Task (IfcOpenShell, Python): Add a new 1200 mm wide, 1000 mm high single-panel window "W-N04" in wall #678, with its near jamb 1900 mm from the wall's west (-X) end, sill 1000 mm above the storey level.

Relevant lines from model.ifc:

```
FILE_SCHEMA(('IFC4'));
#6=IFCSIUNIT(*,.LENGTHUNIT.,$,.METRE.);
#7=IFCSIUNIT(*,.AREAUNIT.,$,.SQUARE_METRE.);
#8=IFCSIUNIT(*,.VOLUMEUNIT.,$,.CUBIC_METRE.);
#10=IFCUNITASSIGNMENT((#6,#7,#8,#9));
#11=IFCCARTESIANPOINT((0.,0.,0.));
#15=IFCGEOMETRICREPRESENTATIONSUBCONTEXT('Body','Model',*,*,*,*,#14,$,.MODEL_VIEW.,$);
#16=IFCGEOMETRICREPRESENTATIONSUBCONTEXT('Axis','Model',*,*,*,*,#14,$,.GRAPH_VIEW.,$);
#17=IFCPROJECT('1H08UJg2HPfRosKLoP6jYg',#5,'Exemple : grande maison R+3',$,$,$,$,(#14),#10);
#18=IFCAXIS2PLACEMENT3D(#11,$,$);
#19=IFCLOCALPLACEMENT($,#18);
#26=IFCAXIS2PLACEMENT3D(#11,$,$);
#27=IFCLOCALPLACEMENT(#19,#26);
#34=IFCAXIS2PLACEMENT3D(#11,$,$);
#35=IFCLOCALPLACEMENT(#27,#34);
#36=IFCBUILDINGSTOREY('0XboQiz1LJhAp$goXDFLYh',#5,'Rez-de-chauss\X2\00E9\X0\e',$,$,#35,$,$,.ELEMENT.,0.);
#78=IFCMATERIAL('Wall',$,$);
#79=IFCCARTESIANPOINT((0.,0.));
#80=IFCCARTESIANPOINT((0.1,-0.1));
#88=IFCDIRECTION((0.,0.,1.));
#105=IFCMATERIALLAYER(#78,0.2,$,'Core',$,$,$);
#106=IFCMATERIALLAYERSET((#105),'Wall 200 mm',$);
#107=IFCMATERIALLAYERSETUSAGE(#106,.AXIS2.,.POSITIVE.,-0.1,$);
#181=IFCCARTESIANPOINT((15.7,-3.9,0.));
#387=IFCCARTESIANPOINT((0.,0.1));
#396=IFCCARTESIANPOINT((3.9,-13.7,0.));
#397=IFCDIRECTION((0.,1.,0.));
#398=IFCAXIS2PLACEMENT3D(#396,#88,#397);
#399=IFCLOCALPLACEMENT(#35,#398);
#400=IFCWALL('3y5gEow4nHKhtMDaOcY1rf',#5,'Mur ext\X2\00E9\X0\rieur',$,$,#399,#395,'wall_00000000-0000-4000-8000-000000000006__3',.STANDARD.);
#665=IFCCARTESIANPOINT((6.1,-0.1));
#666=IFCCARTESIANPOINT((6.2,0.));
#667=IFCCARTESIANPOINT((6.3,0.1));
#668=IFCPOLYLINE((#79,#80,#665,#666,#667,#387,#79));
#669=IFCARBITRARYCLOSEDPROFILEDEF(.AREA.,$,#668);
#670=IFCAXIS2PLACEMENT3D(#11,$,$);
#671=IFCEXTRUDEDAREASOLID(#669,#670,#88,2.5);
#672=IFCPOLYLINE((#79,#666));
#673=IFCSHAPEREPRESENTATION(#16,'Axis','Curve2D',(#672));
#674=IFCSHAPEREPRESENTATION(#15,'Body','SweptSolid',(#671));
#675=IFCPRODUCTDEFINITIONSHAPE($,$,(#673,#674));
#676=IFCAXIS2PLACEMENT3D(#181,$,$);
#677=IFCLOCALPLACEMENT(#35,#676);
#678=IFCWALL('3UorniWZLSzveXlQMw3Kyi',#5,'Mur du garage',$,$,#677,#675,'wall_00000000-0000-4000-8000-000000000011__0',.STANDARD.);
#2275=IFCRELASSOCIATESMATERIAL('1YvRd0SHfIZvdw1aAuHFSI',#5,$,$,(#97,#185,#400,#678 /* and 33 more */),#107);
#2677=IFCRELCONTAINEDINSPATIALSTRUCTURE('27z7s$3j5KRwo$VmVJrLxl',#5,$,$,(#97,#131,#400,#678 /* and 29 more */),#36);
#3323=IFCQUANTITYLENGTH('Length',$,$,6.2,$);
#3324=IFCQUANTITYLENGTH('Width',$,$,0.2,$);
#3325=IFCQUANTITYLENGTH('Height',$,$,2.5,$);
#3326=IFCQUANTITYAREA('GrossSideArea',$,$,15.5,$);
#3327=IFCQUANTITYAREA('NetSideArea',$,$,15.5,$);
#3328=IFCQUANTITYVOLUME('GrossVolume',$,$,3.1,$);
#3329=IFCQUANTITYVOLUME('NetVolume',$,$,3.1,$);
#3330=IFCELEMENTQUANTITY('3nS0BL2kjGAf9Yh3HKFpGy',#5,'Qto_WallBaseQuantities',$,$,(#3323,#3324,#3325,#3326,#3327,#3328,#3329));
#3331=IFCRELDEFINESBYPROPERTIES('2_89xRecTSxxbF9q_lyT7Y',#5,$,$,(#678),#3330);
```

```python
import numpy as np
import ifcopenshell
import ifcopenshell.api.feature
import ifcopenshell.api.geometry
import ifcopenshell.api.pset
import ifcopenshell.api.root
import ifcopenshell.api.spatial
import ifcopenshell.geom
import ifcopenshell.util.element
import ifcopenshell.util.placement
import ifcopenshell.util.representation
import ifcopenshell.util.shape
import ifcopenshell.util.unit

model = ifcopenshell.open("model.ifc")
unit_scale = ifcopenshell.util.unit.calculate_unit_scale(model)
area_scale = ifcopenshell.util.unit.calculate_unit_scale(model, "AREAUNIT")
volume_scale = ifcopenshell.util.unit.calculate_unit_scale(model, "VOLUMEUNIT")
settings = ifcopenshell.geom.settings()


def volume(element):
    """Net volume in cubic metres, openings subtracted."""
    shape = ifcopenshell.geom.create_shape(settings, element)
    return ifcopenshell.util.shape.get_volume(shape.geometry)


wall = model.by_guid("3UorniWZLSzveXlQMw3Kyi")
storey = ifcopenshell.util.element.get_container(wall, ifc_class="IfcBuildingStorey")
context = ifcopenshell.util.representation.get_context(model, "Model", "Body", "MODEL_VIEW")
before = volume(wall)

width, height, from_end, sill = 1.2, 1, 1.9, 1  # metres

# The wall runs along its own X axis, and the end named is its -X end.
wall_shape = ifcopenshell.geom.create_shape(settings, wall)
x, y, z = ifcopenshell.util.shape.get_vertices(wall_shape.geometry).T
start = x.min() + from_end
face, thickness = float(y.min()), float(y.max() - y.min())
wall_matrix = ifcopenshell.util.placement.get_local_placement(wall.ObjectPlacement)
level = ifcopenshell.util.placement.get_local_placement(storey.ObjectPlacement)[2, 3]


def in_wall(x, y):
    """Placement at x, y metres in the wall's axes, at sill height."""
    matrix = wall_matrix.copy()
    matrix[:, 3] = wall_matrix @ np.array([x / unit_scale, y / unit_scale, 0.0, 1.0])
    matrix[2, 3] = level + sill / unit_scale
    return matrix


# Opening: a box that overshoots both wall faces by 50 mm.
opening = ifcopenshell.api.root.create_entity(model, ifc_class="IfcOpeningElement", predefined_type="OPENING")
box = ifcopenshell.api.geometry.add_wall_representation(
    model, context=context, length=width, height=height, thickness=thickness + 0.1
)
ifcopenshell.api.geometry.assign_representation(model, product=opening, representation=box)
ifcopenshell.api.geometry.edit_object_placement(model, product=opening, matrix=in_wall(start, face - 0.05), is_si=False)
ifcopenshell.api.feature.add_feature(model, feature=opening, element=wall)

window = ifcopenshell.api.root.create_entity(model, ifc_class="IfcWindow", name="W-N04", predefined_type="WINDOW")
window.OverallWidth, window.OverallHeight = width / unit_scale, height / unit_scale
window.PartitioningType = "SINGLE_PANEL"
body = ifcopenshell.api.geometry.add_window_representation(
    model,
    context=context,
    overall_width=window.OverallWidth,
    overall_height=window.OverallHeight,
    partition_type="SINGLE_PANEL",
)
ifcopenshell.api.geometry.assign_representation(model, product=window, representation=body)
ifcopenshell.api.spatial.assign_container(model, products=[window], relating_structure=storey)
ifcopenshell.api.feature.add_filling(model, opening=opening, element=window)

# Centre the window in the wall's thickness.
ifcopenshell.api.geometry.edit_object_placement(model, product=window, matrix=in_wall(start, face), is_si=False)
window_shape = ifcopenshell.geom.create_shape(settings, window)
depth = ifcopenshell.util.shape.get_vertices(window_shape.geometry)[:, 1]
offset = face + thickness / 2 - (depth.min() + depth.max()) / 2
ifcopenshell.api.geometry.edit_object_placement(model, product=window, matrix=in_wall(start, offset), is_si=False)

after = volume(wall)

# Update the wall's stored quantities.
qto = model.by_id(ifcopenshell.util.element.get_pset(wall, "Qto_WallBaseQuantities", should_inherit=False)["id"])
ifcopenshell.api.pset.edit_qto(model, qto=qto, properties={
    "NetSideArea": after / thickness / area_scale,
    "NetVolume": after / volume_scale,
})

print(f"wall volume {before:.3f} -> {after:.3f} m3")

model.write("model_v2.ifc")
```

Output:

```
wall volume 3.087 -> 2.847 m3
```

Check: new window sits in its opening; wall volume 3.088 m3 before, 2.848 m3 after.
